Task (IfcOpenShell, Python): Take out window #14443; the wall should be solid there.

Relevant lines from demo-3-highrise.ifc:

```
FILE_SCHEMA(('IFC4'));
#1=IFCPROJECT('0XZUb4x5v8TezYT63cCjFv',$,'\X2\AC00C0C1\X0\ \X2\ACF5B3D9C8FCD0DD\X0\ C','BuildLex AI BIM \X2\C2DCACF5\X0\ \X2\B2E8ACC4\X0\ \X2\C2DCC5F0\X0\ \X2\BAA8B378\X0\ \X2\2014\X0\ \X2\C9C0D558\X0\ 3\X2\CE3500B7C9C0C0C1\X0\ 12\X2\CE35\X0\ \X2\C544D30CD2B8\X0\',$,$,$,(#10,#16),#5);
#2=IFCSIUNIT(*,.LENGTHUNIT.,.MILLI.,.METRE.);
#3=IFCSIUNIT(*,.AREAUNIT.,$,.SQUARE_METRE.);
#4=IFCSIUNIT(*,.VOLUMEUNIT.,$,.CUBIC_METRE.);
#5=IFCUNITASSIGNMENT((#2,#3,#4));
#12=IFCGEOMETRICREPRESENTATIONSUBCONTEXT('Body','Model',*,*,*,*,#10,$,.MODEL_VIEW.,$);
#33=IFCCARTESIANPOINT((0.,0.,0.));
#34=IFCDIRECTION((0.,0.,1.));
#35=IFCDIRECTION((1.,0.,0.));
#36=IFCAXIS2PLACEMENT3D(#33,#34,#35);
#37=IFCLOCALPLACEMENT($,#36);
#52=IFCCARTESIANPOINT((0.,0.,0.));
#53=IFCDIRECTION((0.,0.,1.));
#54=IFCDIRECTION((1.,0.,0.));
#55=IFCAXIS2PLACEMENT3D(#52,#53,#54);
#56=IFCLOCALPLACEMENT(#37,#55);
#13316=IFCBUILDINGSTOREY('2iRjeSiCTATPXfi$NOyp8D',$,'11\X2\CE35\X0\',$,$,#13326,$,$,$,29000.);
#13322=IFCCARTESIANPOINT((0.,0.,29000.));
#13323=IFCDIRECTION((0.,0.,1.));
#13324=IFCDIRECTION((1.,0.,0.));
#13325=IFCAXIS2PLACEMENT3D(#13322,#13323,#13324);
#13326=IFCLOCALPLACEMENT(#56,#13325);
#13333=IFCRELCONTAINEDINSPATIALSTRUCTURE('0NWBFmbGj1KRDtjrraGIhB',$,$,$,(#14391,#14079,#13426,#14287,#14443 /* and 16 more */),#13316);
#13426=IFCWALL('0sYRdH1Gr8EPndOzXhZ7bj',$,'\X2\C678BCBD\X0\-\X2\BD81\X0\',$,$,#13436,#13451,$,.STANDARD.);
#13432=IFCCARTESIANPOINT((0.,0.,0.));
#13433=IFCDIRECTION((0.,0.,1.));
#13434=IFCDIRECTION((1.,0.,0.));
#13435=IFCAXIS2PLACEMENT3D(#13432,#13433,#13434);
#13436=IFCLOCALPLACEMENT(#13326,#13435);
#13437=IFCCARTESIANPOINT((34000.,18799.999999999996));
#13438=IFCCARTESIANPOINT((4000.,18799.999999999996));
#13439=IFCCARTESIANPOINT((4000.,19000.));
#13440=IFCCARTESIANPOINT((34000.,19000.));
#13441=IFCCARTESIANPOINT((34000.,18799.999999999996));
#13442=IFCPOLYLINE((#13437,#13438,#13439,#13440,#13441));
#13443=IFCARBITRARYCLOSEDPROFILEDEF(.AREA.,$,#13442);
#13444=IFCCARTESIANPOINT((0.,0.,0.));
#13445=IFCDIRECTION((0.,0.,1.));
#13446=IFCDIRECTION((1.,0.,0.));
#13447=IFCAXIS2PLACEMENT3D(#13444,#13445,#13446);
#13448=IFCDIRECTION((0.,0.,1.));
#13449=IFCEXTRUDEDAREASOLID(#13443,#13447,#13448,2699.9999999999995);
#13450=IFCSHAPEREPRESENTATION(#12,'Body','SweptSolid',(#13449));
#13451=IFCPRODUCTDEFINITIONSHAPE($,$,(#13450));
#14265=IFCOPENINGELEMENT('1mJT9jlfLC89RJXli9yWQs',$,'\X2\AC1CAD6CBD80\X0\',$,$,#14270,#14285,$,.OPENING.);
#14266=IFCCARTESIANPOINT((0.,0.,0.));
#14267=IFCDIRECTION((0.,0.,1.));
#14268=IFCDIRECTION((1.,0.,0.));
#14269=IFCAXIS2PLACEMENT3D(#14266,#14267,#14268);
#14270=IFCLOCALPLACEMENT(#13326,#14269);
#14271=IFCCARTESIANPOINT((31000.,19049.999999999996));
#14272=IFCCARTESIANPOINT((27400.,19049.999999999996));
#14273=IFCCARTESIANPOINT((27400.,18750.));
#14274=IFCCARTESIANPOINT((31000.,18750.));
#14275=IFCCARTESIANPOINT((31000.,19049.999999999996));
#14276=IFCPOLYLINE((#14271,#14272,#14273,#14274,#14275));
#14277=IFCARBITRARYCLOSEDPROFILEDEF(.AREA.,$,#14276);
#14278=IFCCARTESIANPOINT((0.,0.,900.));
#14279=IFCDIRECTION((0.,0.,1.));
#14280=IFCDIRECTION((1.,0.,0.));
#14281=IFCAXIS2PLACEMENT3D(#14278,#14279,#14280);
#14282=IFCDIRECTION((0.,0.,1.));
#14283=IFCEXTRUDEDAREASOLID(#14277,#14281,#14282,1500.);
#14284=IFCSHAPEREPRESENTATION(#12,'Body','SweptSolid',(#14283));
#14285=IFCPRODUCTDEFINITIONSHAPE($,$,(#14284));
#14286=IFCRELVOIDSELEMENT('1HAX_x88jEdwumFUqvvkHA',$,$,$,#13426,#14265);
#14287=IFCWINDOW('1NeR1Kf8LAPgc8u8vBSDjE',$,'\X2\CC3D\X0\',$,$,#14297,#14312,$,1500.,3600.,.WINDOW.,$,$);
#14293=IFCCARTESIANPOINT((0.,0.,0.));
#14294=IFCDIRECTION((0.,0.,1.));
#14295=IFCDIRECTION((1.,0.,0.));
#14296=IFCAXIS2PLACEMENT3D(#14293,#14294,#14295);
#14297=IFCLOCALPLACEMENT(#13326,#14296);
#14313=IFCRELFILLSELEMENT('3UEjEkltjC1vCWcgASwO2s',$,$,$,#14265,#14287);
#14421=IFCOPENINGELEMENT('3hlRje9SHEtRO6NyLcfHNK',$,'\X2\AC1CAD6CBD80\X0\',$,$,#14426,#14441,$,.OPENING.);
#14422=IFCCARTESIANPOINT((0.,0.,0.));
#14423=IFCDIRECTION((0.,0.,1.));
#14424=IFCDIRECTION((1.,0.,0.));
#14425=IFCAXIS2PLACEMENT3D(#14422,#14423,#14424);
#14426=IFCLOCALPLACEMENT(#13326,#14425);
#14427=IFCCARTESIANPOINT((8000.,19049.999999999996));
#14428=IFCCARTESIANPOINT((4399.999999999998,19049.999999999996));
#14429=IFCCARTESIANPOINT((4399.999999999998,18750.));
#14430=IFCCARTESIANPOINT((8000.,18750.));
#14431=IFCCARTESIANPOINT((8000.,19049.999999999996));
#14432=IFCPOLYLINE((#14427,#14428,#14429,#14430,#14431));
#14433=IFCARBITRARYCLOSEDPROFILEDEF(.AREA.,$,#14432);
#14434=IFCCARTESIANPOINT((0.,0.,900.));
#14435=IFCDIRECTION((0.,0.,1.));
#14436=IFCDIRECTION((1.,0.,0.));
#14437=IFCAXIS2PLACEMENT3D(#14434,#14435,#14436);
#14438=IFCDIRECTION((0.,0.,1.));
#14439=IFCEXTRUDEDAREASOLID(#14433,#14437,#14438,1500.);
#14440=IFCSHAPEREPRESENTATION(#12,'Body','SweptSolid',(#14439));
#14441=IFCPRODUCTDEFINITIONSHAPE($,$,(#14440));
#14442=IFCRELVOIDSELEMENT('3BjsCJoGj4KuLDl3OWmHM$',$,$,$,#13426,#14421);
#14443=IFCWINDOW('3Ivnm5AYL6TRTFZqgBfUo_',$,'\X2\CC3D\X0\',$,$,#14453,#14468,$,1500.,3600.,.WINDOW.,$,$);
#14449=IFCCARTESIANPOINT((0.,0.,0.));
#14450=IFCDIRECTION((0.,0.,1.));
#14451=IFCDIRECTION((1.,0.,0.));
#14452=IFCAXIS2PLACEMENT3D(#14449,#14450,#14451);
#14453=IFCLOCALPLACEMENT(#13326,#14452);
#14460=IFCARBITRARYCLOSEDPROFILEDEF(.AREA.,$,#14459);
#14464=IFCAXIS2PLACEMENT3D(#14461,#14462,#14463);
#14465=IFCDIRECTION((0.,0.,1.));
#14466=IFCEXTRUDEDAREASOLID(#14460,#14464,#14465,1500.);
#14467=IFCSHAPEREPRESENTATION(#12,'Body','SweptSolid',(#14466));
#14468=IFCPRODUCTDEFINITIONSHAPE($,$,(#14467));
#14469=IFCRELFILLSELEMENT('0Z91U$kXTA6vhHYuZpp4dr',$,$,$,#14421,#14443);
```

```python
import ifcopenshell
import ifcopenshell.api.feature
import ifcopenshell.api.root
import ifcopenshell.geom
import ifcopenshell.util.shape

model = ifcopenshell.open("demo-3-highrise.ifc")
settings = ifcopenshell.geom.settings()


def volume(element):
    """Net volume in cubic metres, openings subtracted."""
    shape = ifcopenshell.geom.create_shape(settings, element)
    return ifcopenshell.util.shape.get_volume(shape.geometry)


window = model.by_guid("3Ivnm5AYL6TRTFZqgBfUo_")
opening = window.FillsVoids[0].RelatingOpeningElement
wall = opening.VoidsElements[0].RelatingBuildingElement
before = volume(wall)

ifcopenshell.api.root.remove_product(model, product=window)
ifcopenshell.api.feature.remove_feature(model, feature=opening)

after = volume(wall)

print(f"wall volume {before:.3f} -> {after:.3f} m3")

model.write("demo-3-highrise_edited.ifc")
```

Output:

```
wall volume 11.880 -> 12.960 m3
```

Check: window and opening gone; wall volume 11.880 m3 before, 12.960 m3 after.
